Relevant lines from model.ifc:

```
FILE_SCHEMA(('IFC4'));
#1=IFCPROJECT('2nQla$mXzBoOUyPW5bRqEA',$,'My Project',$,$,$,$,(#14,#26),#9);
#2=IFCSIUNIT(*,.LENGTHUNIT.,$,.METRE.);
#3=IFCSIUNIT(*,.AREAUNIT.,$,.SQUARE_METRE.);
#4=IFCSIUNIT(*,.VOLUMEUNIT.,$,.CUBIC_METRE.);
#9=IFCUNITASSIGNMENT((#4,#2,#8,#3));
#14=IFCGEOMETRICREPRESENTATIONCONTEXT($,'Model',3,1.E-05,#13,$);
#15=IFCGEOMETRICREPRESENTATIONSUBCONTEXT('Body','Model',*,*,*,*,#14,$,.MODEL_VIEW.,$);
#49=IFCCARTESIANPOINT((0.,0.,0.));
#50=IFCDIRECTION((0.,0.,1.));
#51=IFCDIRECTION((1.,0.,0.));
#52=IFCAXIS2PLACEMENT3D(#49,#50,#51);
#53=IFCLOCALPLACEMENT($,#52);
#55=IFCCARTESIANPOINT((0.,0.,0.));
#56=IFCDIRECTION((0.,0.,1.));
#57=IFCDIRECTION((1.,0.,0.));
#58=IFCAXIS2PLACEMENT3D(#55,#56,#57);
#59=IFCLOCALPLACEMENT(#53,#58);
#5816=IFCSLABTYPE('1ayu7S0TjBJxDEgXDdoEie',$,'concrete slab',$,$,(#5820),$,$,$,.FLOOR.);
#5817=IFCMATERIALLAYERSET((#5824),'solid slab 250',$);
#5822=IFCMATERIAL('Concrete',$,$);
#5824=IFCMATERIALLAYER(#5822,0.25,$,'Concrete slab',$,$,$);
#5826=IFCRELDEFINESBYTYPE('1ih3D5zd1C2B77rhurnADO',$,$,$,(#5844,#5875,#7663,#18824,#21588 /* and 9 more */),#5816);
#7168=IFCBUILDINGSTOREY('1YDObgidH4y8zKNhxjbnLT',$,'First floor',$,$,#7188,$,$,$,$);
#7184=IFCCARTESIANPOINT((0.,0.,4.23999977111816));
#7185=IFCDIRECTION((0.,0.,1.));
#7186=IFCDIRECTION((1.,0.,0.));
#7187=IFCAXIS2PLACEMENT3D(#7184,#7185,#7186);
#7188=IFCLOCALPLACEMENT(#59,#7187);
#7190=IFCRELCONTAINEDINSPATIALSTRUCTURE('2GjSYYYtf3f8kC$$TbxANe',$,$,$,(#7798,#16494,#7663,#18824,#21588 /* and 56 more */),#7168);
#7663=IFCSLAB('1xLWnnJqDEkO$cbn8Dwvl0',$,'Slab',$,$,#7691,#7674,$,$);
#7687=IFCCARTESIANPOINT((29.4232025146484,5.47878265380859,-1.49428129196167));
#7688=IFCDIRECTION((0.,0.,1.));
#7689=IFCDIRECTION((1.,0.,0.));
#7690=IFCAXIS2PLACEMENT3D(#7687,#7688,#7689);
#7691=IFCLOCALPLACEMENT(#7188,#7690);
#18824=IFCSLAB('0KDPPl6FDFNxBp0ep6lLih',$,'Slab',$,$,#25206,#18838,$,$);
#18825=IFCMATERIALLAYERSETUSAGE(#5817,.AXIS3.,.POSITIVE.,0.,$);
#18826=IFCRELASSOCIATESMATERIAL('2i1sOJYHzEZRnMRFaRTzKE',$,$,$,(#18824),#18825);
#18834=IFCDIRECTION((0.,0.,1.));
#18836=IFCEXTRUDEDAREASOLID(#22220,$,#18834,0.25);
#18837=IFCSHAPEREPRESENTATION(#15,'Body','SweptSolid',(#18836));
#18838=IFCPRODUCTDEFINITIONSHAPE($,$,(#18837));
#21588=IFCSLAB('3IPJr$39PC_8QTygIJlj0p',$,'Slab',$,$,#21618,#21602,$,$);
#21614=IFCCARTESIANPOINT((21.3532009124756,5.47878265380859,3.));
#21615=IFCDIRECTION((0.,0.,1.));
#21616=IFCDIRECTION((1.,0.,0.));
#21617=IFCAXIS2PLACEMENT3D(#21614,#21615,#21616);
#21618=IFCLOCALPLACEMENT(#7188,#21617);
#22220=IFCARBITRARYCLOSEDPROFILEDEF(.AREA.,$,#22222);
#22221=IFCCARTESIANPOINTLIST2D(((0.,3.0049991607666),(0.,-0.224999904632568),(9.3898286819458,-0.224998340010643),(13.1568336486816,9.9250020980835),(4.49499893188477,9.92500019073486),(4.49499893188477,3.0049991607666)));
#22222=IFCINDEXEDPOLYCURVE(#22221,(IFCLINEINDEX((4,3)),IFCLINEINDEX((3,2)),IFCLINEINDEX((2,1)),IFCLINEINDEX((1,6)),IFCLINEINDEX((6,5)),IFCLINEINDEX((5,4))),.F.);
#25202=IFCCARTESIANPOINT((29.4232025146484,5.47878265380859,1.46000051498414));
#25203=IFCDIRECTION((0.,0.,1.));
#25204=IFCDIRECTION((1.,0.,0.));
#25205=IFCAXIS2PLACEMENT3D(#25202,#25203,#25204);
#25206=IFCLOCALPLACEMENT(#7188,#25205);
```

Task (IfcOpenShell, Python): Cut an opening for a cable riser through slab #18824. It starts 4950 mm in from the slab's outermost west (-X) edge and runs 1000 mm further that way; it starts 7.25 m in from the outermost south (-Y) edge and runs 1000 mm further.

```python
import numpy as np
import ifcopenshell
import ifcopenshell.api.feature
import ifcopenshell.api.geometry
import ifcopenshell.api.root
import ifcopenshell.geom
import ifcopenshell.util.placement
import ifcopenshell.util.representation
import ifcopenshell.util.shape
import ifcopenshell.util.unit

model = ifcopenshell.open("model.ifc")
unit_scale = ifcopenshell.util.unit.calculate_unit_scale(model)
settings = ifcopenshell.geom.settings()


def volume(element):
    """Net volume in cubic metres, openings subtracted."""
    shape = ifcopenshell.geom.create_shape(settings, element)
    return ifcopenshell.util.shape.get_volume(shape.geometry)


slab = model.by_guid("0KDPPl6FDFNxBp0ep6lLih")
before = volume(slab)

# Extent in the slab's own axes, in metres. The edges named are its -X and -Y sides.
slab_shape = ifcopenshell.geom.create_shape(settings, slab)
vertices = ifcopenshell.util.shape.get_vertices(slab_shape.geometry)
x_min, y_min, bottom = vertices.min(axis=0)
top = vertices[:, 2].max()

opening = ifcopenshell.api.root.create_entity(model, ifc_class="IfcOpeningElement", name="Cable riser opening", predefined_type="OPENING")
context = ifcopenshell.util.representation.get_context(model, "Model", "Body", "MODEL_VIEW")
width, depth = 1, 1
outline = [(0.0, 0.0), (width, 0.0), (width, depth), (0.0, depth), (0.0, 0.0)]
# Overshoot both faces by 50 mm so the cut is clean.
shape = ifcopenshell.api.geometry.add_slab_representation(
    model, context=context, depth=top - bottom + 0.1, polyline=outline
)
ifcopenshell.api.geometry.assign_representation(model, product=opening, representation=shape)

matrix = ifcopenshell.util.placement.get_local_placement(slab.ObjectPlacement)
matrix[:, 3] = matrix @ np.append(np.array([x_min + 4.95, y_min + 7.25, bottom - 0.05]) / unit_scale, 1.0)
ifcopenshell.api.geometry.edit_object_placement(model, product=opening, matrix=matrix, is_si=False)
ifcopenshell.api.feature.add_feature(model, feature=opening, element=slab)

after = volume(slab)

print(f"slab volume {before:.3f} -> {after:.3f} m3")

model.write("model_edited.ifc")
```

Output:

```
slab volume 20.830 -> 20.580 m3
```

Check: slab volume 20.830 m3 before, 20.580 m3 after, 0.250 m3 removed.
